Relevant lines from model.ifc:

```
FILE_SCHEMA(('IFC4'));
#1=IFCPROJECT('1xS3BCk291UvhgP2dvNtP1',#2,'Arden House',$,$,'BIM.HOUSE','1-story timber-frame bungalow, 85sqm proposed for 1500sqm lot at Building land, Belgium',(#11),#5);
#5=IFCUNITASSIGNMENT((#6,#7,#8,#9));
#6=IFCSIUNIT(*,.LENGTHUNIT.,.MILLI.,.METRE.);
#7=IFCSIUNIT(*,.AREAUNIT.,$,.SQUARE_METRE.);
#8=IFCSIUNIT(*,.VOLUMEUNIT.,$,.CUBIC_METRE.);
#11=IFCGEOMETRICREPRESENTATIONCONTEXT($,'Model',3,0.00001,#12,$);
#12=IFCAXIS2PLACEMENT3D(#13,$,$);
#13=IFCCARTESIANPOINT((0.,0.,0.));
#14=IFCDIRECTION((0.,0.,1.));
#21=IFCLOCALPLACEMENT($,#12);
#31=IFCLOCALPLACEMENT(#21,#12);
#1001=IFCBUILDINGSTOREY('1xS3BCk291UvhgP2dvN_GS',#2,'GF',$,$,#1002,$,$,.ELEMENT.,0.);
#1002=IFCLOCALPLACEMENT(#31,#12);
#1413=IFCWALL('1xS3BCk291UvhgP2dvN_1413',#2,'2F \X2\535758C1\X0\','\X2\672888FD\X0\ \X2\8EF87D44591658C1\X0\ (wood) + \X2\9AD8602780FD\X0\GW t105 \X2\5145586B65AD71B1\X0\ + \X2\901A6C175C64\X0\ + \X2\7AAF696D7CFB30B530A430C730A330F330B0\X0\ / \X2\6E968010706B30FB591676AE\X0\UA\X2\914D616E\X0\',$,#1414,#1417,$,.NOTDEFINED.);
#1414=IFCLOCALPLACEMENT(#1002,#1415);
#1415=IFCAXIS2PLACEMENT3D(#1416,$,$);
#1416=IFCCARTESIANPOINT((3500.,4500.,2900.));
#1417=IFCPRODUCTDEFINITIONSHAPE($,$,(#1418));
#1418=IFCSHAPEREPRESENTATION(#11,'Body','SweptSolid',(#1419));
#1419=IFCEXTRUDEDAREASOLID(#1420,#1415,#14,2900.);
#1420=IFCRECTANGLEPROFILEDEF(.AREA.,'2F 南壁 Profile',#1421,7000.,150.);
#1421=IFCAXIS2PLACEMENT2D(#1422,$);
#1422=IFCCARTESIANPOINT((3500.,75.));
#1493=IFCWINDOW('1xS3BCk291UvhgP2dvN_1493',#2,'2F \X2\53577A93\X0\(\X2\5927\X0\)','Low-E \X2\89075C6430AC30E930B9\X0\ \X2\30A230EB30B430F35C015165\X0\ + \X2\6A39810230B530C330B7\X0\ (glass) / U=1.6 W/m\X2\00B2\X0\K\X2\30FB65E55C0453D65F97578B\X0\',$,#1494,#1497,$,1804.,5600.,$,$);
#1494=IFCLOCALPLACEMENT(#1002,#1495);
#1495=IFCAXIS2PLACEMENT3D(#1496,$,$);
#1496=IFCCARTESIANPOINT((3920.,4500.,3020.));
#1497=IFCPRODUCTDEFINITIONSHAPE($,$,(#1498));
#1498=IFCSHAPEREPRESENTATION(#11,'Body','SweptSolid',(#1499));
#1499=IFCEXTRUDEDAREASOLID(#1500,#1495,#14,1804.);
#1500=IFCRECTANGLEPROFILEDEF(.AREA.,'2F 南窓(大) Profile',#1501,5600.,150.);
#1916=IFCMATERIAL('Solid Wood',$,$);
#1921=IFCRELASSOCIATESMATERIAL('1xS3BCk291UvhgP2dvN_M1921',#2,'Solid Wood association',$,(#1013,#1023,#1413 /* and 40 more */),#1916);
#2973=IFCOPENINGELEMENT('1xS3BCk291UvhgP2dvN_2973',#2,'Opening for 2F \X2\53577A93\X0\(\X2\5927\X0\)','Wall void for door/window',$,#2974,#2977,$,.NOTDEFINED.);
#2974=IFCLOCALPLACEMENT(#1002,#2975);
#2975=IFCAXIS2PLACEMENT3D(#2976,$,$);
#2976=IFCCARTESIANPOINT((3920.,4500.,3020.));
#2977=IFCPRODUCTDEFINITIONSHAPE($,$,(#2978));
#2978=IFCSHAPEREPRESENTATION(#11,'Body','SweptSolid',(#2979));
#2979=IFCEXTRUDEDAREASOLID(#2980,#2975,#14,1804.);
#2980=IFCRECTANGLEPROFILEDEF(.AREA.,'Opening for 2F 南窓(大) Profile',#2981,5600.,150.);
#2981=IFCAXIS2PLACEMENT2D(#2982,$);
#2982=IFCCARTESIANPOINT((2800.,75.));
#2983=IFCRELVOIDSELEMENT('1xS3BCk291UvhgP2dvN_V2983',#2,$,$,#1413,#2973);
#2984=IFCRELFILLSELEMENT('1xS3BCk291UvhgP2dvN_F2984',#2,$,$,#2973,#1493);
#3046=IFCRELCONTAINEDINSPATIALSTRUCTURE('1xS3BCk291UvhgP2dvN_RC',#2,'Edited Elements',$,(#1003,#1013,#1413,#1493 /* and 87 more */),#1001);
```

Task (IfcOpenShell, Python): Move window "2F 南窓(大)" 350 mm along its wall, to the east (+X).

```python
import ifcopenshell
import ifcopenshell.api.geometry
import ifcopenshell.util.placement
import ifcopenshell.util.unit

model = ifcopenshell.open("model.ifc")
unit_scale = ifcopenshell.util.unit.calculate_unit_scale(model)

window = model.by_guid("1xS3BCk291UvhgP2dvN_1493")
opening = window.FillsVoids[0].RelatingOpeningElement
wall = opening.VoidsElements[0].RelatingBuildingElement

wall_matrix = ifcopenshell.util.placement.get_local_placement(wall.ObjectPlacement)
shift = wall_matrix[:3, 0] * 0.35 / unit_scale
before = ifcopenshell.util.placement.get_local_placement(window.ObjectPlacement)[:3, 3].copy()

# The window is not placed relative to its opening, so move both.
for product in (opening, window):
    matrix = ifcopenshell.util.placement.get_local_placement(product.ObjectPlacement)
    matrix[:3, 3] += shift
    ifcopenshell.api.geometry.edit_object_placement(model, product=product, matrix=matrix, is_si=False)

after = ifcopenshell.util.placement.get_local_placement(window.ObjectPlacement)[:3, 3]
print("window moved by", (after - before).round(3) + 0.0)

model.write("model_updated.ifc")
```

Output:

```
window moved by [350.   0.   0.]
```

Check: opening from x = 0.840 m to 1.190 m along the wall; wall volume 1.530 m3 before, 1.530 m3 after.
